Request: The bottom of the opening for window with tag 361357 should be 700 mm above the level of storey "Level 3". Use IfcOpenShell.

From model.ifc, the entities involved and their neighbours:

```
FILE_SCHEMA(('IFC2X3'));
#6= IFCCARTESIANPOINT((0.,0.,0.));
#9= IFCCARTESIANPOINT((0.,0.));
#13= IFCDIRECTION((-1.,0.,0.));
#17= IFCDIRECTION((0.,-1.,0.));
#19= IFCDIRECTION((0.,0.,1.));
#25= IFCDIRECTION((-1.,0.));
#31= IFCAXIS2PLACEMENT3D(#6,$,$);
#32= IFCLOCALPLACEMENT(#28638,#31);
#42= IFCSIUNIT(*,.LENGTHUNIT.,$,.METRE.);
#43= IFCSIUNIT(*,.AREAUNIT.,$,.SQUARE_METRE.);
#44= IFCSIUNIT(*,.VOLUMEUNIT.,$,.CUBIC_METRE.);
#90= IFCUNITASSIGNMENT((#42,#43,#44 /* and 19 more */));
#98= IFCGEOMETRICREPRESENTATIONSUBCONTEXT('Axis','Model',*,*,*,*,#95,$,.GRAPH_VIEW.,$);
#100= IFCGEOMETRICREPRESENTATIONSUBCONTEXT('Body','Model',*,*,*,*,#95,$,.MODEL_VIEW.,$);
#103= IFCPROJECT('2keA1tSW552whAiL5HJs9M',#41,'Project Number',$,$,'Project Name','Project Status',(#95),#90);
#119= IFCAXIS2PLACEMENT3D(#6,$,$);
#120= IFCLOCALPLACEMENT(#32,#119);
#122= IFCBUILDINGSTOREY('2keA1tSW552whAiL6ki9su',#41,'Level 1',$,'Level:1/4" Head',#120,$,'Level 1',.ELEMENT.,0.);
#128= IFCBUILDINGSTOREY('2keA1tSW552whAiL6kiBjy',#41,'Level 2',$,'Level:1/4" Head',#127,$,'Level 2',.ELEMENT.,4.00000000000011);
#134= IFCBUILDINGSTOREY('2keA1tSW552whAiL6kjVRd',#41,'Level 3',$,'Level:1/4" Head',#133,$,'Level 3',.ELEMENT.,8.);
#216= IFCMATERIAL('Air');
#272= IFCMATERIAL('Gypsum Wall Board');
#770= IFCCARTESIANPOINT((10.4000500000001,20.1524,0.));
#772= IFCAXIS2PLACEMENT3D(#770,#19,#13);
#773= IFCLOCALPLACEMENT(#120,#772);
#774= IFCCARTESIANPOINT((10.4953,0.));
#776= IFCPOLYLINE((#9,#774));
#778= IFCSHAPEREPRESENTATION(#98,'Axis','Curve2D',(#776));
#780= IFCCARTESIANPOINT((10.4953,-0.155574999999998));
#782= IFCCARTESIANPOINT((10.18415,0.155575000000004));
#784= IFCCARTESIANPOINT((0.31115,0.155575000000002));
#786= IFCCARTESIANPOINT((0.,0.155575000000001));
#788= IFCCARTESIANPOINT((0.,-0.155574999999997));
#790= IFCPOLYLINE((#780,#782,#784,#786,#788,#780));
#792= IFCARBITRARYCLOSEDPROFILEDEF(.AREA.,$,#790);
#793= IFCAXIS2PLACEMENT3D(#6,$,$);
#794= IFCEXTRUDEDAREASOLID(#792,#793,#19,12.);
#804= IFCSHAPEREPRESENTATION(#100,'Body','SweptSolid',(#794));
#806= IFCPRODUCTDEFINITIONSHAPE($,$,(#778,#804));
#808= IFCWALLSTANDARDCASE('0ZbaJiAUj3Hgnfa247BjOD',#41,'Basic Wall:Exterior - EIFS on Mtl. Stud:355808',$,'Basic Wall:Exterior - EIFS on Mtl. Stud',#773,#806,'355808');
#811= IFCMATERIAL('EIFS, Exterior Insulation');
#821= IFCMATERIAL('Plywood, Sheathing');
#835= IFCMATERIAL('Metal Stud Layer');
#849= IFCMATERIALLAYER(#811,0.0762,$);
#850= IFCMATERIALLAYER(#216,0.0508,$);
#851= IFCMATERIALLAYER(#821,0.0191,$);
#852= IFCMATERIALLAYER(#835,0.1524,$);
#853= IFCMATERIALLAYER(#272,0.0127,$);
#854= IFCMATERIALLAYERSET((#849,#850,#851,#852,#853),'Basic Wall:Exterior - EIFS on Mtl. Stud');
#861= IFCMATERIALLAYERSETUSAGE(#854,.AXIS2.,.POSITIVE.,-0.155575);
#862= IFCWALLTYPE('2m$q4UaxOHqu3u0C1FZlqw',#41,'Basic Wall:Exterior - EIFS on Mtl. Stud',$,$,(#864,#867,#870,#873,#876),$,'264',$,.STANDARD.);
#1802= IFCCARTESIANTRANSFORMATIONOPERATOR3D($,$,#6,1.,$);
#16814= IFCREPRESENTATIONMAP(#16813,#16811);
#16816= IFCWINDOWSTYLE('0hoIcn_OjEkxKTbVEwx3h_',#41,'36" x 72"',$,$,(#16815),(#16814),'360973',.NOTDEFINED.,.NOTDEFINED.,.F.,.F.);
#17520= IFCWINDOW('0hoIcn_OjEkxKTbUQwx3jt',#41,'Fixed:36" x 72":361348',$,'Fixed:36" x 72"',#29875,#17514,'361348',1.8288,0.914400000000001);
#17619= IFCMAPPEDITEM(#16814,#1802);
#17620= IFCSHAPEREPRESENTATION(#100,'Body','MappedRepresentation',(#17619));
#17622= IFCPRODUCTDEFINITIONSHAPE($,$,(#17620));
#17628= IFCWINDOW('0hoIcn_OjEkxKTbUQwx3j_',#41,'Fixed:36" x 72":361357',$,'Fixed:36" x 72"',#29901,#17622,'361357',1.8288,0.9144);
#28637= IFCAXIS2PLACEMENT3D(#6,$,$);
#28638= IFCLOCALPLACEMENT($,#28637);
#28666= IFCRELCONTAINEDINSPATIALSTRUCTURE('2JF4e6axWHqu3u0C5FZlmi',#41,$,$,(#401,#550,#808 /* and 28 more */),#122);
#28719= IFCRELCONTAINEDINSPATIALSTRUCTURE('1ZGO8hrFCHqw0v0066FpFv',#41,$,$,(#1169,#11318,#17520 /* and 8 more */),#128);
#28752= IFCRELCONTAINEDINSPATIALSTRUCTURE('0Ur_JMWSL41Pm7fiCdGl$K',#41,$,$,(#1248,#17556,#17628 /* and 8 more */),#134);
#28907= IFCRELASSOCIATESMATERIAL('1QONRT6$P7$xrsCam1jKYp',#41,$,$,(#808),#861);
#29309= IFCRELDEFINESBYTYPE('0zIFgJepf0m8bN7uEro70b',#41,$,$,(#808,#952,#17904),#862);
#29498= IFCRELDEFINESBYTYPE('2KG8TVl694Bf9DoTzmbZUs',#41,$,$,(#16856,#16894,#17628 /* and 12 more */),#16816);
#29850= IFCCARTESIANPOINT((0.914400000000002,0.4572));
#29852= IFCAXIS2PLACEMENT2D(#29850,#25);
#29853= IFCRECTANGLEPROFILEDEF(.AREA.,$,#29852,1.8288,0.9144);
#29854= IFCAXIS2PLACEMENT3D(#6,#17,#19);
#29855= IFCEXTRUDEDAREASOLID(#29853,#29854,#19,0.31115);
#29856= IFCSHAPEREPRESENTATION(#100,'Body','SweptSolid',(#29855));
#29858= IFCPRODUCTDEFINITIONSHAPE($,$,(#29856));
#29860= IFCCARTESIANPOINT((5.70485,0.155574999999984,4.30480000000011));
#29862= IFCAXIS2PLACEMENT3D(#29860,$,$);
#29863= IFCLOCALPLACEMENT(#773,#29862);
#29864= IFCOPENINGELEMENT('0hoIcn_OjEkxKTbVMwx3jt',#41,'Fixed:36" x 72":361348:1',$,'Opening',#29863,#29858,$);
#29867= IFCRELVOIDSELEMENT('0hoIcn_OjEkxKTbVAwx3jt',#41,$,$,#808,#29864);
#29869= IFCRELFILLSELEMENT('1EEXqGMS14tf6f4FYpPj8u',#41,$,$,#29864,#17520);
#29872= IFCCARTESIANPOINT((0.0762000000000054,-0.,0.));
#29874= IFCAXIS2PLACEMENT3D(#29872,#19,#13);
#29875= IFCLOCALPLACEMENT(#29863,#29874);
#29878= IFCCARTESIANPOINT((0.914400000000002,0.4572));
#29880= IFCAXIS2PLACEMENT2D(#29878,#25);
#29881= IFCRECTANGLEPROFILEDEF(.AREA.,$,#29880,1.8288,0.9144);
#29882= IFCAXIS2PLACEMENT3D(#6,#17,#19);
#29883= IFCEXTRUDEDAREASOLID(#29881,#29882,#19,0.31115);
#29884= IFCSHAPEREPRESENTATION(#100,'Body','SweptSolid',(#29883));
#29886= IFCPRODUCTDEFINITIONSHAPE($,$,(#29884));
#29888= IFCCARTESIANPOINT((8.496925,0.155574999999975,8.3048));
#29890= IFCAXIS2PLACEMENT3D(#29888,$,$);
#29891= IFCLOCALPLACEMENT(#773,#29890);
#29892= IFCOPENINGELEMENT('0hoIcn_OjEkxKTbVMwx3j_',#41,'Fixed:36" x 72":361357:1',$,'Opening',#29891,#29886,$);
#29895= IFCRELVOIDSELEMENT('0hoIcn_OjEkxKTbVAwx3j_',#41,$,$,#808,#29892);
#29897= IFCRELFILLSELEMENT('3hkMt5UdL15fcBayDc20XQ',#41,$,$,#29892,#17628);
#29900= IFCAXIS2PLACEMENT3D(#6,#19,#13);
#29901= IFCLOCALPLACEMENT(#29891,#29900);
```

```python
import numpy as np
import ifcopenshell
import ifcopenshell.api.geometry
import ifcopenshell.geom
import ifcopenshell.util.element
import ifcopenshell.util.placement
import ifcopenshell.util.shape
import ifcopenshell.util.unit

model = ifcopenshell.open("model.ifc")
unit_scale = ifcopenshell.util.unit.calculate_unit_scale(model)

window = model.by_id(17628)
opening = window.FillsVoids[0].RelatingOpeningElement
storey = ifcopenshell.util.element.get_container(window, ifc_class="IfcBuildingStorey")
level = ifcopenshell.util.placement.get_local_placement(storey.ObjectPlacement)[2, 3]

# The opening's origin need not be at the sill, so measure its lowest point.
shape = ifcopenshell.geom.create_shape(ifcopenshell.geom.settings(), opening)
bottom = ifcopenshell.util.shape.get_shape_bottom_elevation(shape, shape.geometry) / unit_scale
dz = level + 0.7 / unit_scale - bottom

shift = np.array([0.0, 0.0, dz])
# The window is placed relative to its opening, so it follows when the opening moves.
matrix = ifcopenshell.util.placement.get_local_placement(opening.ObjectPlacement)
matrix[:3, 3] += shift
ifcopenshell.api.geometry.edit_object_placement(
    model, product=opening, matrix=matrix, is_si=False, should_transform_children=True
)

print(f"moved by {dz * unit_scale:+.3f} m")

model.write("model_edited.ifc")
```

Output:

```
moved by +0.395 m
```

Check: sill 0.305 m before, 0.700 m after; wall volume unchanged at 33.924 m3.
